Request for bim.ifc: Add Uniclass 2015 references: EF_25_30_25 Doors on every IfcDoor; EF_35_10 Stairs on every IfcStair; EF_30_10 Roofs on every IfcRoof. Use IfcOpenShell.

First a look at what the model holds.

```python
import ifcopenshell

model = ifcopenshell.open("bim.ifc")
print(model.schema)
print("classifications:", [c.Name for c in model.by_type("IfcClassification")])
for ifc_class in ("IfcDoor", "IfcRoof", "IfcStair", "IfcWall", "IfcWindow"):
    print(ifc_class, len(model.by_type(ifc_class)))
```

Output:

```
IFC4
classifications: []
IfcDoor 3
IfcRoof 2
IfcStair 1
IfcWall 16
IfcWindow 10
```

```python
import ifcopenshell
import ifcopenshell.api.classification

model = ifcopenshell.open("bim.ifc")

system = ifcopenshell.api.classification.add_classification(model, classification="Uniclass 2015")

codes = {
    "IfcDoor": ("EF_25_30_25", "Doors"),
    "IfcStair": ("EF_35_10", "Stairs"),
    "IfcRoof": ("EF_30_10", "Roofs"),
}
for ifc_class, (code, name) in codes.items():
    products = model.by_type(ifc_class)
    ifcopenshell.api.classification.add_reference(
        model, products=products, classification=system, identification=code, name=name
    )
    print(code, len(products))

model.write("bim_rev.ifc")
```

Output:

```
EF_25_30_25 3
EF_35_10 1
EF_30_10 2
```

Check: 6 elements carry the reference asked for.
